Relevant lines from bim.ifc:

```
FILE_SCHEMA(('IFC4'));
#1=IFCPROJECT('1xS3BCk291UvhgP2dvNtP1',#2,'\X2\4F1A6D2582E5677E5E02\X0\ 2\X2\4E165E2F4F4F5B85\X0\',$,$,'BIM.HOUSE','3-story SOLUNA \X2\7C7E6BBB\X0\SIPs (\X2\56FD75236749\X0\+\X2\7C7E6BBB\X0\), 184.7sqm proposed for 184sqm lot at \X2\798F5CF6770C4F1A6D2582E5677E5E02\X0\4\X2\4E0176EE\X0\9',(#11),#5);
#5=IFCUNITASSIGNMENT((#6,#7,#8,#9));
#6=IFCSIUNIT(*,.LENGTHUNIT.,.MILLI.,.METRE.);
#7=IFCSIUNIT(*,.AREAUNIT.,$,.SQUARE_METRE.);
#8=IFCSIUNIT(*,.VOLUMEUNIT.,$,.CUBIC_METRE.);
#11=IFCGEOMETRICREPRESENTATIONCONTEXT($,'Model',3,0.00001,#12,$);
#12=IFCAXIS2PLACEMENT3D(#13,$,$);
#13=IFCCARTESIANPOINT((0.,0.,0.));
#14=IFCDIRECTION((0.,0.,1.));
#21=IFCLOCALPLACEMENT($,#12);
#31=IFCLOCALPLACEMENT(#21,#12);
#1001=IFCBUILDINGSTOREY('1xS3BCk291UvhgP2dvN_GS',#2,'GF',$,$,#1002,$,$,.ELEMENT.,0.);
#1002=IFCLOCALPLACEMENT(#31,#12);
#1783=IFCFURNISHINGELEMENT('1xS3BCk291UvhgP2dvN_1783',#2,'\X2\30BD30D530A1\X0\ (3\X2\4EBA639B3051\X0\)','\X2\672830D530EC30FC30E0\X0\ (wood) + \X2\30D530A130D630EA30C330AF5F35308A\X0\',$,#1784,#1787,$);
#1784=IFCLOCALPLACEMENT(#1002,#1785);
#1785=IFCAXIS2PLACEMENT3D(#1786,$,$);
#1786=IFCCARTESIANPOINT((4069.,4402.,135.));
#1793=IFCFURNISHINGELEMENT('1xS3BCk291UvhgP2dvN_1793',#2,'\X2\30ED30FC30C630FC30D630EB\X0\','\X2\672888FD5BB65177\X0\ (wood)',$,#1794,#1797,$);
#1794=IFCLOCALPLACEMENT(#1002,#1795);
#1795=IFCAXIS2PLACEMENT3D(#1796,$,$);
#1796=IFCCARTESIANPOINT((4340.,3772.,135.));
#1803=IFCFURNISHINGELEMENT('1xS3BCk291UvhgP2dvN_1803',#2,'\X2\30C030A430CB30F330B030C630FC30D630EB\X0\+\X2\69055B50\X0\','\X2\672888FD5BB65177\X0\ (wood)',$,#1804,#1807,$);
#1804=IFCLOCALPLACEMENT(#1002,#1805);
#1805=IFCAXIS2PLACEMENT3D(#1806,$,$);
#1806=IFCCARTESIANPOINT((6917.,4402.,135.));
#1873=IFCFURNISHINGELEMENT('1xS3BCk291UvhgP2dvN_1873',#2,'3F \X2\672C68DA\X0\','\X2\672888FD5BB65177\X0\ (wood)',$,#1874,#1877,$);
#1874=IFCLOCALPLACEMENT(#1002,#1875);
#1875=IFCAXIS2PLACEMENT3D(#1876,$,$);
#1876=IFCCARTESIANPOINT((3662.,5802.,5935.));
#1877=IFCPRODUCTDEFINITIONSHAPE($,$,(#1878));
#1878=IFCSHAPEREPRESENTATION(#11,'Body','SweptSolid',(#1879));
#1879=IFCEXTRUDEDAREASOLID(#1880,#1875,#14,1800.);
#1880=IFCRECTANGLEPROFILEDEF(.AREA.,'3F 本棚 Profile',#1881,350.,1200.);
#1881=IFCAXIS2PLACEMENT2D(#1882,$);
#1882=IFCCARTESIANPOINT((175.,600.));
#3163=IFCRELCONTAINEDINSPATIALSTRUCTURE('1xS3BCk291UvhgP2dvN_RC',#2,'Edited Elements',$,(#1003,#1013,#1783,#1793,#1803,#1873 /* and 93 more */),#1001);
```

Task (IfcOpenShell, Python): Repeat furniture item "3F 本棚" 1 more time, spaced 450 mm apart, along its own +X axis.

```python
import ifcopenshell
import ifcopenshell.api.geometry
import ifcopenshell.api.root
import ifcopenshell.util.element
import ifcopenshell.util.placement

model = ifcopenshell.open("bim.ifc")


def reuse_history(source, copy):
    """copy_class also copies each property set's owner history, people and application; keep the originals."""
    for rel in copy.IsDefinedBy:
        if rel.is_a("IfcRelDefinesByProperties") and (history := rel.RelatingPropertyDefinition.OwnerHistory):
            rel.RelatingPropertyDefinition.OwnerHistory = source.OwnerHistory
            ifcopenshell.util.element.remove_deep2(model, history)


source = model.by_guid("1xS3BCk291UvhgP2dvN_1873")
base = ifcopenshell.util.placement.get_local_placement(source.ObjectPlacement)
step = base[:3, 0] * 450.0

for i in range(1, 2):
    copy = ifcopenshell.api.root.copy_class(model, product=source)
    copy.Representation = ifcopenshell.util.element.copy_deep(
        model, source.Representation, exclude=["IfcGeometricRepresentationContext", "IfcRepresentationMap"]
    )
    reuse_history(source, copy)
    matrix = base.copy()
    matrix[:3, 3] += i * step
    print("added at", matrix[:3, 3].round(3) + 0.0)
    ifcopenshell.api.geometry.edit_object_placement(model, product=copy, matrix=matrix, is_si=False)

model.write("bim_updated.ifc")
```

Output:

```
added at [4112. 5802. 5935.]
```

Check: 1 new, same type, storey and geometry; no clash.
